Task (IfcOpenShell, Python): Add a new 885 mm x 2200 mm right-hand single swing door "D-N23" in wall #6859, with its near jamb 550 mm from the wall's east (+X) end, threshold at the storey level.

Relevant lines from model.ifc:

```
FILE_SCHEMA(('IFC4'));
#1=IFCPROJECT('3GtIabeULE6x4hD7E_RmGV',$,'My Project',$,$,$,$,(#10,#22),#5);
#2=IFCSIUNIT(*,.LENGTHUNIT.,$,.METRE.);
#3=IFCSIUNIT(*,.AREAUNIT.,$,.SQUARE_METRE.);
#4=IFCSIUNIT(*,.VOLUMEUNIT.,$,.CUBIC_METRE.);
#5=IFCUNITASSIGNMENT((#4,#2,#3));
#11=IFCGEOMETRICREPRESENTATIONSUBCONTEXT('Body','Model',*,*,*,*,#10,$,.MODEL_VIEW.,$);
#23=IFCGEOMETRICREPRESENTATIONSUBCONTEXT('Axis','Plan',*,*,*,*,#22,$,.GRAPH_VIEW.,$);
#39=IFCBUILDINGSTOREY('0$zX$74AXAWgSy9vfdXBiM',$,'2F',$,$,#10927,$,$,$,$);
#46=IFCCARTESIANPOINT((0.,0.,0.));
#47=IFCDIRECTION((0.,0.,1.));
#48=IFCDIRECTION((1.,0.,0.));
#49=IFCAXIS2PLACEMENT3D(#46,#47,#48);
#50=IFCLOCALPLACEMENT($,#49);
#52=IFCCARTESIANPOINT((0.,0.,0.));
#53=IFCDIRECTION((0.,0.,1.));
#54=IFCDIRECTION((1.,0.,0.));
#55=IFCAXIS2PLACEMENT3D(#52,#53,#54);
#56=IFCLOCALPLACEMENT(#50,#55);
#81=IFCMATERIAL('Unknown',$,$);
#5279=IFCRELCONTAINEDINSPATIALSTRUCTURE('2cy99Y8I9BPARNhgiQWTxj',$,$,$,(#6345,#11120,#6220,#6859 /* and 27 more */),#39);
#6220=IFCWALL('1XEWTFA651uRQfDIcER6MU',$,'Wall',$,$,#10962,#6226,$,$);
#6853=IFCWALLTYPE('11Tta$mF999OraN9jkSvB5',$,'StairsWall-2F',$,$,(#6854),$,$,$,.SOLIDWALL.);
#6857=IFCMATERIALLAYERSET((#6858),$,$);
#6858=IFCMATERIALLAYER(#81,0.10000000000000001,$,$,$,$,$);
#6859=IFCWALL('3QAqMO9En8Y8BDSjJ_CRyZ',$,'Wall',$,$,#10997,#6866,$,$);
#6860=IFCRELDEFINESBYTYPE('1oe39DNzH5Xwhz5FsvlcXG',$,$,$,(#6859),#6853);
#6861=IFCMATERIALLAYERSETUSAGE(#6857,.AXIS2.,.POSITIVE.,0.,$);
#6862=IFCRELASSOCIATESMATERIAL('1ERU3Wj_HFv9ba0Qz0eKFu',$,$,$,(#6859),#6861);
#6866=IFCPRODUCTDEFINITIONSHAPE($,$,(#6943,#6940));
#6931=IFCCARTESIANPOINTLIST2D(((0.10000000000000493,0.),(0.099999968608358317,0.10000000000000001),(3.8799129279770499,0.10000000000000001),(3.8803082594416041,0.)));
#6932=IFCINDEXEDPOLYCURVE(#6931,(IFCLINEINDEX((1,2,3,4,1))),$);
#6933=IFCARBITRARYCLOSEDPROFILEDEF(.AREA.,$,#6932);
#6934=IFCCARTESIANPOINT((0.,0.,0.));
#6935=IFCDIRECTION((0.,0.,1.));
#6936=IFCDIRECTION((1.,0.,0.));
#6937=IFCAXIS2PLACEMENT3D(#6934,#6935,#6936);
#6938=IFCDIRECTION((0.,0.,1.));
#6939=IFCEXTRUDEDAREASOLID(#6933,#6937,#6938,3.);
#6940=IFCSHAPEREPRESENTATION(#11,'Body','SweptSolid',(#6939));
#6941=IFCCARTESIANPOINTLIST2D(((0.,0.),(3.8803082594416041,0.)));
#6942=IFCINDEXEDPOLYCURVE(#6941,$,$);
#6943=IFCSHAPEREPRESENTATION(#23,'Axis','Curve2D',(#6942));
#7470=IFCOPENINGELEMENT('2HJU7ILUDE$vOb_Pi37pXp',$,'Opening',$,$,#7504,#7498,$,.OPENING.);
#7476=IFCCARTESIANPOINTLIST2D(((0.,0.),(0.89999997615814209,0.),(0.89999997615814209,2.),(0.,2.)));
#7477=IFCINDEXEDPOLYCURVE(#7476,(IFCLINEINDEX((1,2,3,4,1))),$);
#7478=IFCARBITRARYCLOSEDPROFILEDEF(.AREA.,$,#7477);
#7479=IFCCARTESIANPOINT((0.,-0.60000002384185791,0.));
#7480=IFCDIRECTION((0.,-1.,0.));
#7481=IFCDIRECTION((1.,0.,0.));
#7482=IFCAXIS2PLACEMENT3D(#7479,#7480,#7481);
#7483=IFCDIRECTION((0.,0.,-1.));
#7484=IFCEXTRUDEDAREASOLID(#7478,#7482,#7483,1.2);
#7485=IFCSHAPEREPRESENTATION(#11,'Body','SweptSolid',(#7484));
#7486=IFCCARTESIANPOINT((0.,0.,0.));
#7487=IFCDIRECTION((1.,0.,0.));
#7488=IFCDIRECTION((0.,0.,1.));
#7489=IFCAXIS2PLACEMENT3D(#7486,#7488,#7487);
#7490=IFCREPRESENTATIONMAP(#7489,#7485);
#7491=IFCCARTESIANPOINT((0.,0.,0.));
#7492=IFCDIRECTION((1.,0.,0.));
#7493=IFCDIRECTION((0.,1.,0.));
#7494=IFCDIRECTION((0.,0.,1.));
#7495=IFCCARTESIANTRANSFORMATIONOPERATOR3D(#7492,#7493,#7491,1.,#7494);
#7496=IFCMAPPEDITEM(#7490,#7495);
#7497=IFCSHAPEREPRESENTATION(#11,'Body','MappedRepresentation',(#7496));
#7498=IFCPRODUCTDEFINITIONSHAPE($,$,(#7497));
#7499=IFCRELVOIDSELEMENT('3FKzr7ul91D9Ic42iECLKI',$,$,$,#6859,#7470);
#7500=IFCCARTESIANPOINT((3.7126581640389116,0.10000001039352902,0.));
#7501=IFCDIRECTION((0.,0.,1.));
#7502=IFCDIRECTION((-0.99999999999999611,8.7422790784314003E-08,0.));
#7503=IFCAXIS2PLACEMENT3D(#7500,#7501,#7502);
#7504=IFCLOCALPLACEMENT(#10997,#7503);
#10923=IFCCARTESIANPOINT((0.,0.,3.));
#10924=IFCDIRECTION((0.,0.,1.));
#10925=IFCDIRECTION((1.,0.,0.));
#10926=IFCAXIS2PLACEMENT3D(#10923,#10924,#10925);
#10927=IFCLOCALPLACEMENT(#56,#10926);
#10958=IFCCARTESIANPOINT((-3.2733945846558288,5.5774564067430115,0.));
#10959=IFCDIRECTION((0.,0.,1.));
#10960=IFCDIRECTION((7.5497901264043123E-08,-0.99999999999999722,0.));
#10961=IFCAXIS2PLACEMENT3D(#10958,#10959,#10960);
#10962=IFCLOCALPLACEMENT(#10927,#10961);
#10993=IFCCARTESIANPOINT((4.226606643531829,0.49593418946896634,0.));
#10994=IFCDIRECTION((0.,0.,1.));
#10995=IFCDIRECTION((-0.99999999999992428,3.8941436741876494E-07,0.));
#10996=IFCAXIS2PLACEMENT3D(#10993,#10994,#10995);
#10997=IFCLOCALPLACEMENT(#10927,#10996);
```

```python
import numpy as np
import ifcopenshell
import ifcopenshell.api.feature
import ifcopenshell.api.geometry
import ifcopenshell.api.root
import ifcopenshell.api.spatial
import ifcopenshell.geom
import ifcopenshell.util.element
import ifcopenshell.util.placement
import ifcopenshell.util.representation
import ifcopenshell.util.shape
import ifcopenshell.util.unit

model = ifcopenshell.open("model.ifc")
unit_scale = ifcopenshell.util.unit.calculate_unit_scale(model)
settings = ifcopenshell.geom.settings()


def volume(element):
    """Net volume in cubic metres, openings subtracted."""
    shape = ifcopenshell.geom.create_shape(settings, element)
    return ifcopenshell.util.shape.get_volume(shape.geometry)


wall = model.by_guid("3QAqMO9En8Y8BDSjJ_CRyZ")
storey = ifcopenshell.util.element.get_container(wall, ifc_class="IfcBuildingStorey")
context = ifcopenshell.util.representation.get_context(model, "Model", "Body", "MODEL_VIEW")
before = volume(wall)

width, height, from_end, sill = 0.885, 2.2, 0.55, 0.0  # metres

# The wall runs along its own X axis, and the end named is its -X end.
wall_shape = ifcopenshell.geom.create_shape(settings, wall)
x, y, z = ifcopenshell.util.shape.get_vertices(wall_shape.geometry).T
start = x.min() + from_end
face, thickness = float(y.min()), float(y.max() - y.min())
wall_matrix = ifcopenshell.util.placement.get_local_placement(wall.ObjectPlacement)
level = ifcopenshell.util.placement.get_local_placement(storey.ObjectPlacement)[2, 3]


def in_wall(x, y):
    """Placement at x, y metres in the wall's axes, at sill height."""
    matrix = wall_matrix.copy()
    matrix[:, 3] = wall_matrix @ np.array([x / unit_scale, y / unit_scale, 0.0, 1.0])
    matrix[2, 3] = level + sill / unit_scale
    return matrix


# Opening: a box that overshoots both wall faces by 50 mm.
opening = ifcopenshell.api.root.create_entity(model, ifc_class="IfcOpeningElement", predefined_type="OPENING")
box = ifcopenshell.api.geometry.add_wall_representation(
    model, context=context, length=width, height=height, thickness=thickness + 0.1
)
ifcopenshell.api.geometry.assign_representation(model, product=opening, representation=box)
ifcopenshell.api.geometry.edit_object_placement(model, product=opening, matrix=in_wall(start, face - 0.05), is_si=False)
ifcopenshell.api.feature.add_feature(model, feature=opening, element=wall)

door = ifcopenshell.api.root.create_entity(model, ifc_class="IfcDoor", name="D-N23", predefined_type="DOOR")
door.OverallWidth, door.OverallHeight = width / unit_scale, height / unit_scale
door.OperationType = "SINGLE_SWING_RIGHT"
body = ifcopenshell.api.geometry.add_door_representation(
    model,
    context=context,
    overall_width=door.OverallWidth,
    overall_height=door.OverallHeight,
    operation_type="SINGLE_SWING_RIGHT",
    lining_properties={"LiningDepth": thickness / unit_scale, "ThresholdDepth": thickness / unit_scale},
)
ifcopenshell.api.geometry.assign_representation(model, product=door, representation=body)
ifcopenshell.api.spatial.assign_container(model, products=[door], relating_structure=storey)
ifcopenshell.api.feature.add_filling(model, opening=opening, element=door)

# The lining spans the wall, so the door starts at the wall face.
ifcopenshell.api.geometry.edit_object_placement(model, product=door, matrix=in_wall(start, face), is_si=False)

after = volume(wall)

print(f"wall volume {before:.3f} -> {after:.3f} m3")

model.write("model_edited.ifc")
```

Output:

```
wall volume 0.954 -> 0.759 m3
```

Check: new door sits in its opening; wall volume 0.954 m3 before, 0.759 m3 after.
